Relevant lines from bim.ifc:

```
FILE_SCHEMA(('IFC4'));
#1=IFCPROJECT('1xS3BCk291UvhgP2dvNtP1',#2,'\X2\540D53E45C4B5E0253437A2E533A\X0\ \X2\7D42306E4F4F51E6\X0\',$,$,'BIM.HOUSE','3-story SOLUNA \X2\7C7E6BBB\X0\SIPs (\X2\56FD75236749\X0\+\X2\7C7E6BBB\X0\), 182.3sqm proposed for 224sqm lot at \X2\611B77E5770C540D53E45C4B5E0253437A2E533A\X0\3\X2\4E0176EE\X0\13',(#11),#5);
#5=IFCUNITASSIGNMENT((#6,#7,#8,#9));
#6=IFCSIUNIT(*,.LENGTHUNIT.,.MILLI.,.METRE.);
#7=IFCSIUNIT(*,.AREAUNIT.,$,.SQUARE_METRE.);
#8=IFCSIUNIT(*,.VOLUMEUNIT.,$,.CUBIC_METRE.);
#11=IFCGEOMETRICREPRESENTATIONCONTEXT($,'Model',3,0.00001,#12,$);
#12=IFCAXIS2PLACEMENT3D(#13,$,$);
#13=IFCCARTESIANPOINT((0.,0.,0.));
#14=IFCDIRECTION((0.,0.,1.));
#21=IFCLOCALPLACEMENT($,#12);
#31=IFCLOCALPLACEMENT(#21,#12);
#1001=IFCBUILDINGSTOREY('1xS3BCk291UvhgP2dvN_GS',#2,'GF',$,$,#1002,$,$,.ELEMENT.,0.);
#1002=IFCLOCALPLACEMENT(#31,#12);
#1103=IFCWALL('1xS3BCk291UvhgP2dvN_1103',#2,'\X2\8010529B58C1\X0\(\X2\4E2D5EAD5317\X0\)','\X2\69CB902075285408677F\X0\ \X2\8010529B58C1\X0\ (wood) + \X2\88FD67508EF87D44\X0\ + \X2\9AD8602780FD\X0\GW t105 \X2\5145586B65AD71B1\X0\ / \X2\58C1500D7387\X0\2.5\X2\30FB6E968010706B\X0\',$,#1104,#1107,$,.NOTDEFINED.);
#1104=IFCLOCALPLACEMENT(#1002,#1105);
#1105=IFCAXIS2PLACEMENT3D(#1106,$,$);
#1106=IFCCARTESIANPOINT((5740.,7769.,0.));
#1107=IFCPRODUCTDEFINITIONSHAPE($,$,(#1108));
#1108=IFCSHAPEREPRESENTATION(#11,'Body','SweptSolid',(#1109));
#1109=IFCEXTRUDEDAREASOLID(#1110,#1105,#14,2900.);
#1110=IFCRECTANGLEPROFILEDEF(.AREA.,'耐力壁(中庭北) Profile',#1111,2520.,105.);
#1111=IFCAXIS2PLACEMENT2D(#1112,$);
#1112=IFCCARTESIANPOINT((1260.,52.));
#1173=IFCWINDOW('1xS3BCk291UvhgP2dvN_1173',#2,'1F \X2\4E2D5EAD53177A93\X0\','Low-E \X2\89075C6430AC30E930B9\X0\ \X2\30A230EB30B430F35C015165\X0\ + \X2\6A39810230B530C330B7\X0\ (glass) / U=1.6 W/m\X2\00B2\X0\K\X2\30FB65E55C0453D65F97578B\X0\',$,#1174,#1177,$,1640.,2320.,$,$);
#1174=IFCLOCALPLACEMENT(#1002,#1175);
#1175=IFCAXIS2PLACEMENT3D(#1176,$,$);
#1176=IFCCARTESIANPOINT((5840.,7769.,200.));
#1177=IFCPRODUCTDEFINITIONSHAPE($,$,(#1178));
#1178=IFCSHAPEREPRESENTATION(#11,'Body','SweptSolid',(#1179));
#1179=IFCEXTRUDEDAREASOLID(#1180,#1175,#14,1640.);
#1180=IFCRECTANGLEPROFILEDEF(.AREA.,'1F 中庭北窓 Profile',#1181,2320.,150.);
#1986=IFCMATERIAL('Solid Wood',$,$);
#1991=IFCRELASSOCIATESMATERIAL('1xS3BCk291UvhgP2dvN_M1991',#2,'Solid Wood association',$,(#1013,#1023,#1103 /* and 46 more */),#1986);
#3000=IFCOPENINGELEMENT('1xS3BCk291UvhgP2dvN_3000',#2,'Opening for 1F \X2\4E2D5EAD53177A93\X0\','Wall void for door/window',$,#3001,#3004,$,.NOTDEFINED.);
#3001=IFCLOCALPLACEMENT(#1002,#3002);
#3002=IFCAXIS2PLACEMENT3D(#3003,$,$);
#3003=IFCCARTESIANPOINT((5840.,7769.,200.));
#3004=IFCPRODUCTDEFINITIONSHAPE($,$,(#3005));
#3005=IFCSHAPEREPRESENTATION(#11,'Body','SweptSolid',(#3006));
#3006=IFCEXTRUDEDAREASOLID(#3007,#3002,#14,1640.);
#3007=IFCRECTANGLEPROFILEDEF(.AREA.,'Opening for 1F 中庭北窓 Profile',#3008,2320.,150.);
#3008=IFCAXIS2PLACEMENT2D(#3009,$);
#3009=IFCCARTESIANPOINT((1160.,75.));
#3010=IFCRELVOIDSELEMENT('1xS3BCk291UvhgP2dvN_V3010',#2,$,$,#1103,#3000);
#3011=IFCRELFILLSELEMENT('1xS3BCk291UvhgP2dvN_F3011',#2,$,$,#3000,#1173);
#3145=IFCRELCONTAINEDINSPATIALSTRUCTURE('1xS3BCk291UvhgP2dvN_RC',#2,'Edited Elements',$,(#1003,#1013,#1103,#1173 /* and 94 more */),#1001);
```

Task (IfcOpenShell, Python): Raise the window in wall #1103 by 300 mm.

```python
import numpy as np
import ifcopenshell
import ifcopenshell.api.geometry
import ifcopenshell.util.placement
import ifcopenshell.util.unit

model = ifcopenshell.open("bim.ifc")
unit_scale = ifcopenshell.util.unit.calculate_unit_scale(model)

window = model.by_id(1173)
opening = window.FillsVoids[0].RelatingOpeningElement
dz = 300.0

shift = np.array([0.0, 0.0, dz])
# The window is not placed relative to its opening, so move both.
for product in (opening, window):
    matrix = ifcopenshell.util.placement.get_local_placement(product.ObjectPlacement)
    matrix[:3, 3] += shift
    ifcopenshell.api.geometry.edit_object_placement(model, product=product, matrix=matrix, is_si=False)

print(f"moved by {dz * unit_scale:+.3f} m")

model.write("bim_updated.ifc")
```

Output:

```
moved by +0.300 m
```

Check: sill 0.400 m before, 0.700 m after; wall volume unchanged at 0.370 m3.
